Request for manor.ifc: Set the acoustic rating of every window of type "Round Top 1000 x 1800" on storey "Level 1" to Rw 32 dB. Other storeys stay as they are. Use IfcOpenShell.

First a look at what the model holds.

```python
import ifcopenshell
import ifcopenshell.util.element

model = ifcopenshell.open("manor.ifc")
print(model.schema)
storey = next(s for s in model.by_type("IfcBuildingStorey") if s.Name == "Level 1")
windows = [e for e in ifcopenshell.util.element.get_decomposition(storey) if e.is_a("IfcWindow")]
seen = {}
for e in windows:
    element_type = ifcopenshell.util.element.get_type(e)
    key = (element_type.Name if element_type != e and element_type else None, ifcopenshell.util.element.get_pset(e, "Pset_WindowCommon", "AcousticRating"))
    seen[key] = seen.get(key, 0) + 1
for (name, value), count in sorted(seen.items(), key=str):
    print(count, "x", name, "|", value)
```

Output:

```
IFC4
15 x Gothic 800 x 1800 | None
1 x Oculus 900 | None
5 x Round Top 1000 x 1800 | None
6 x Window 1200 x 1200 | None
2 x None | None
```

```python
import ifcopenshell
import ifcopenshell.api.pset
import ifcopenshell.util.element

model = ifcopenshell.open("manor.ifc")

storey = next(s for s in model.by_type("IfcBuildingStorey") if s.Name == "Level 1")
windows = [e for e in ifcopenshell.util.element.get_decomposition(storey) if e.is_a("IfcWindow")]

count = 0
for e in windows:
    element_type = ifcopenshell.util.element.get_type(e)
    if element_type in (None, e) or element_type.Name != "Round Top 1000 x 1800":
        continue
    # add_pset returns the element's existing set when there is one.
    pset = ifcopenshell.api.pset.add_pset(model, product=e, name="Pset_WindowCommon")
    ifcopenshell.api.pset.edit_pset(model, pset=pset, properties={"AcousticRating": "Rw 32 dB"})
    count += 1

print(count, "windows updated")

model.write("manor_v2.ifc")
```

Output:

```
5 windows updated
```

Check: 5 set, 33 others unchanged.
